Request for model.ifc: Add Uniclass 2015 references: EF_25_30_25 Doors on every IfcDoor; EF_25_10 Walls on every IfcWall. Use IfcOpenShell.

First a look at what the model holds.

```python
import ifcopenshell

model = ifcopenshell.open("model.ifc")
print(model.schema)
print("classifications:", [c.Name for c in model.by_type("IfcClassification")])
for ifc_class in ("IfcDoor", "IfcRoof", "IfcStair", "IfcWall", "IfcWindow"):
    print(ifc_class, len(model.by_type(ifc_class)))
```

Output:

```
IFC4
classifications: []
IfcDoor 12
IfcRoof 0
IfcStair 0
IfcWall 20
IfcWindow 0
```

```python
import ifcopenshell
import ifcopenshell.api.classification

model = ifcopenshell.open("model.ifc")

system = ifcopenshell.api.classification.add_classification(model, classification="Uniclass 2015")

codes = {
    "IfcDoor": ("EF_25_30_25", "Doors"),
    "IfcWall": ("EF_25_10", "Walls"),
}
for ifc_class, (code, name) in codes.items():
    products = model.by_type(ifc_class)
    ifcopenshell.api.classification.add_reference(
        model, products=products, classification=system, identification=code, name=name
    )
    print(code, len(products))

model.write("model-out.ifc")
```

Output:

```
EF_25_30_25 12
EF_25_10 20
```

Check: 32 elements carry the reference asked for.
